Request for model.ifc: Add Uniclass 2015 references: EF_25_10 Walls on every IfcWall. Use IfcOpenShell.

First a look at what the model holds.

```python
import ifcopenshell

model = ifcopenshell.open("model.ifc")
print(model.schema)
print("classifications:", [c.Name for c in model.by_type("IfcClassification")])
for ifc_class in ("IfcDoor", "IfcRoof", "IfcStair", "IfcWall", "IfcWindow"):
    print(ifc_class, len(model.by_type(ifc_class)))
```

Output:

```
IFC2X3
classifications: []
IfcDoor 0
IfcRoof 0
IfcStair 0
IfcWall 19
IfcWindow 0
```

```python
import ifcopenshell
import ifcopenshell.api.classification

model = ifcopenshell.open("model.ifc")

# IFC2X3 requires Source and Edition and has no link from the project to the system.
system = model.create_entity("IfcClassification", Source="NBS", Edition="2015", Name="Uniclass 2015")

codes = {
    "IfcWall": ("EF_25_10", "Walls"),
}
for ifc_class, (code, name) in codes.items():
    products = model.by_type(ifc_class)
    ifcopenshell.api.classification.add_reference(
        model, products=products, classification=system, identification=code, name=name
    )
    print(code, len(products))

model.write("model_edited.ifc")
```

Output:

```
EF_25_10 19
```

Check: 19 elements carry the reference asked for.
